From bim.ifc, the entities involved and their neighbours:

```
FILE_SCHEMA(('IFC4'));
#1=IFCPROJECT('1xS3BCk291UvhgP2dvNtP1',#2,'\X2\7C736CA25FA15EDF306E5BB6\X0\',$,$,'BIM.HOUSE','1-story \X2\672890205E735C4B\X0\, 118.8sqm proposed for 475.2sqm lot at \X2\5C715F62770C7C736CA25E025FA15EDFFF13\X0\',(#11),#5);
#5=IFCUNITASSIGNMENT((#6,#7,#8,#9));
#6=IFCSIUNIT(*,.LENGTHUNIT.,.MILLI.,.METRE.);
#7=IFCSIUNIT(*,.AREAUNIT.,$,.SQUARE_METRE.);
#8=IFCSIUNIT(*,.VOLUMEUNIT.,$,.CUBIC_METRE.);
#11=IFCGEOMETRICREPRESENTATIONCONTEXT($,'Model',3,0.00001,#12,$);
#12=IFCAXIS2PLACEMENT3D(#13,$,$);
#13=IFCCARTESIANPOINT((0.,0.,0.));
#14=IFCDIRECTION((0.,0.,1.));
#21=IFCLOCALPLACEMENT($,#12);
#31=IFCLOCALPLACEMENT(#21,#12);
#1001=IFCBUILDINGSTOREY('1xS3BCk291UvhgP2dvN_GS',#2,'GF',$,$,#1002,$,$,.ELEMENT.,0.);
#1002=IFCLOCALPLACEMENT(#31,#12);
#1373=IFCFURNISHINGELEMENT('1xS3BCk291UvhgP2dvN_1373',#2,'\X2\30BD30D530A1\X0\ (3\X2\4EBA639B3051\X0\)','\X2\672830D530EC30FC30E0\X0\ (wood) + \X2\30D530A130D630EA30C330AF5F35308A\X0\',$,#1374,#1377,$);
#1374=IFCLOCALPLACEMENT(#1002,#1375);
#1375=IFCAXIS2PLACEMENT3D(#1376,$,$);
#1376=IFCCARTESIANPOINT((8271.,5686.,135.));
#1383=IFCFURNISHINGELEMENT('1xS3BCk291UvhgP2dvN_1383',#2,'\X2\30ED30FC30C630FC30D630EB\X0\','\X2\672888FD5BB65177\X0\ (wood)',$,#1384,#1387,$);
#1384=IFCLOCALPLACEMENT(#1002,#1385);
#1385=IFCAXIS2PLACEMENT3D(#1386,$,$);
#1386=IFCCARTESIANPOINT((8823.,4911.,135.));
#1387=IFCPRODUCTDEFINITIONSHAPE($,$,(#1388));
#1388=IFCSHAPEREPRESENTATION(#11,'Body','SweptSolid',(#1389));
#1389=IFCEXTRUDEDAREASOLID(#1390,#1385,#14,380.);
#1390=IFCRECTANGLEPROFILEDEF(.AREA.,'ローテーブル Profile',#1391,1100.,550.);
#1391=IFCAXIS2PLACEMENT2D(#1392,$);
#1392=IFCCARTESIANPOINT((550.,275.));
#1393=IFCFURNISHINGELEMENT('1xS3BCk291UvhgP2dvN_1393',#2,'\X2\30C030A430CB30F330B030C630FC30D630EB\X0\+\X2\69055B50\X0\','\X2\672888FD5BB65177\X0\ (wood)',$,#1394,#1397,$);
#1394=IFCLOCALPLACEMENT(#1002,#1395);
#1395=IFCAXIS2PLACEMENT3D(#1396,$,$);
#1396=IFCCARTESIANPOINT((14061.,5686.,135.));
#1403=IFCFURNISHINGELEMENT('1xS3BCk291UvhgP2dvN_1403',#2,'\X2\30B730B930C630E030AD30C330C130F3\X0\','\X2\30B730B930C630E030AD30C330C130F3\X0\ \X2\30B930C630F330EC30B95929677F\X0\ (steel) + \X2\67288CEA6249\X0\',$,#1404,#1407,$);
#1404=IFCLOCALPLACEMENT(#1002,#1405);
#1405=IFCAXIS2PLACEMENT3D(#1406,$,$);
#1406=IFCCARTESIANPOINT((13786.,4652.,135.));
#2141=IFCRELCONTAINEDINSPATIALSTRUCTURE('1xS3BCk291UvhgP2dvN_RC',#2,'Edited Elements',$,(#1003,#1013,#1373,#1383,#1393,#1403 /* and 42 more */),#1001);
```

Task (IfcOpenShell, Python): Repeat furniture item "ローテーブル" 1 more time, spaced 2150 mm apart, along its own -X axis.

```python
import ifcopenshell
import ifcopenshell.api.geometry
import ifcopenshell.api.root
import ifcopenshell.util.element
import ifcopenshell.util.placement
import ifcopenshell.util.unit

model = ifcopenshell.open("bim.ifc")
unit_scale = ifcopenshell.util.unit.calculate_unit_scale(model)


def reuse_history(source, copy):
    """copy_class also copies each property set's owner history, people and application; keep the originals."""
    for rel in copy.IsDefinedBy:
        if rel.is_a("IfcRelDefinesByProperties") and (history := rel.RelatingPropertyDefinition.OwnerHistory):
            rel.RelatingPropertyDefinition.OwnerHistory = source.OwnerHistory
            ifcopenshell.util.element.remove_deep2(model, history)


source = model.by_id(1383)
base = ifcopenshell.util.placement.get_local_placement(source.ObjectPlacement)
step = -base[:3, 0] * 2.15 / unit_scale

for i in range(1, 2):
    copy = ifcopenshell.api.root.copy_class(model, product=source)
    copy.Representation = ifcopenshell.util.element.copy_deep(
        model, source.Representation, exclude=["IfcGeometricRepresentationContext", "IfcRepresentationMap"]
    )
    reuse_history(source, copy)
    matrix = base.copy()
    matrix[:3, 3] += i * step
    print("added at", matrix[:3, 3].round(3) + 0.0)
    ifcopenshell.api.geometry.edit_object_placement(model, product=copy, matrix=matrix, is_si=False)

model.write("bim_v2.ifc")
```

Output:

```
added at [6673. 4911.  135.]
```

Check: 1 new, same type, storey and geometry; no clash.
